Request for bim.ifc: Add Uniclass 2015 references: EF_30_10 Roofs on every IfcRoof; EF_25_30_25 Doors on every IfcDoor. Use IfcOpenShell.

First a look at what the model holds.

```python
import ifcopenshell

model = ifcopenshell.open("bim.ifc")
print(model.schema)
print("classifications:", [c.Name for c in model.by_type("IfcClassification")])
for ifc_class in ("IfcDoor", "IfcRoof", "IfcStair", "IfcWall", "IfcWindow"):
    print(ifc_class, len(model.by_type(ifc_class)))
```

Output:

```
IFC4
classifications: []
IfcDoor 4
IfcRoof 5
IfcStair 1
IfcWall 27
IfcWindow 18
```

```python
import ifcopenshell
import ifcopenshell.api.classification

model = ifcopenshell.open("bim.ifc")

system = ifcopenshell.api.classification.add_classification(model, classification="Uniclass 2015")

codes = {
    "IfcRoof": ("EF_30_10", "Roofs"),
    "IfcDoor": ("EF_25_30_25", "Doors"),
}
for ifc_class, (code, name) in codes.items():
    products = model.by_type(ifc_class)
    ifcopenshell.api.classification.add_reference(
        model, products=products, classification=system, identification=code, name=name
    )
    print(code, len(products))

model.write("bim_updated.ifc")
```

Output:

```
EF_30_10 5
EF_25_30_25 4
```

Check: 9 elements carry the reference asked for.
